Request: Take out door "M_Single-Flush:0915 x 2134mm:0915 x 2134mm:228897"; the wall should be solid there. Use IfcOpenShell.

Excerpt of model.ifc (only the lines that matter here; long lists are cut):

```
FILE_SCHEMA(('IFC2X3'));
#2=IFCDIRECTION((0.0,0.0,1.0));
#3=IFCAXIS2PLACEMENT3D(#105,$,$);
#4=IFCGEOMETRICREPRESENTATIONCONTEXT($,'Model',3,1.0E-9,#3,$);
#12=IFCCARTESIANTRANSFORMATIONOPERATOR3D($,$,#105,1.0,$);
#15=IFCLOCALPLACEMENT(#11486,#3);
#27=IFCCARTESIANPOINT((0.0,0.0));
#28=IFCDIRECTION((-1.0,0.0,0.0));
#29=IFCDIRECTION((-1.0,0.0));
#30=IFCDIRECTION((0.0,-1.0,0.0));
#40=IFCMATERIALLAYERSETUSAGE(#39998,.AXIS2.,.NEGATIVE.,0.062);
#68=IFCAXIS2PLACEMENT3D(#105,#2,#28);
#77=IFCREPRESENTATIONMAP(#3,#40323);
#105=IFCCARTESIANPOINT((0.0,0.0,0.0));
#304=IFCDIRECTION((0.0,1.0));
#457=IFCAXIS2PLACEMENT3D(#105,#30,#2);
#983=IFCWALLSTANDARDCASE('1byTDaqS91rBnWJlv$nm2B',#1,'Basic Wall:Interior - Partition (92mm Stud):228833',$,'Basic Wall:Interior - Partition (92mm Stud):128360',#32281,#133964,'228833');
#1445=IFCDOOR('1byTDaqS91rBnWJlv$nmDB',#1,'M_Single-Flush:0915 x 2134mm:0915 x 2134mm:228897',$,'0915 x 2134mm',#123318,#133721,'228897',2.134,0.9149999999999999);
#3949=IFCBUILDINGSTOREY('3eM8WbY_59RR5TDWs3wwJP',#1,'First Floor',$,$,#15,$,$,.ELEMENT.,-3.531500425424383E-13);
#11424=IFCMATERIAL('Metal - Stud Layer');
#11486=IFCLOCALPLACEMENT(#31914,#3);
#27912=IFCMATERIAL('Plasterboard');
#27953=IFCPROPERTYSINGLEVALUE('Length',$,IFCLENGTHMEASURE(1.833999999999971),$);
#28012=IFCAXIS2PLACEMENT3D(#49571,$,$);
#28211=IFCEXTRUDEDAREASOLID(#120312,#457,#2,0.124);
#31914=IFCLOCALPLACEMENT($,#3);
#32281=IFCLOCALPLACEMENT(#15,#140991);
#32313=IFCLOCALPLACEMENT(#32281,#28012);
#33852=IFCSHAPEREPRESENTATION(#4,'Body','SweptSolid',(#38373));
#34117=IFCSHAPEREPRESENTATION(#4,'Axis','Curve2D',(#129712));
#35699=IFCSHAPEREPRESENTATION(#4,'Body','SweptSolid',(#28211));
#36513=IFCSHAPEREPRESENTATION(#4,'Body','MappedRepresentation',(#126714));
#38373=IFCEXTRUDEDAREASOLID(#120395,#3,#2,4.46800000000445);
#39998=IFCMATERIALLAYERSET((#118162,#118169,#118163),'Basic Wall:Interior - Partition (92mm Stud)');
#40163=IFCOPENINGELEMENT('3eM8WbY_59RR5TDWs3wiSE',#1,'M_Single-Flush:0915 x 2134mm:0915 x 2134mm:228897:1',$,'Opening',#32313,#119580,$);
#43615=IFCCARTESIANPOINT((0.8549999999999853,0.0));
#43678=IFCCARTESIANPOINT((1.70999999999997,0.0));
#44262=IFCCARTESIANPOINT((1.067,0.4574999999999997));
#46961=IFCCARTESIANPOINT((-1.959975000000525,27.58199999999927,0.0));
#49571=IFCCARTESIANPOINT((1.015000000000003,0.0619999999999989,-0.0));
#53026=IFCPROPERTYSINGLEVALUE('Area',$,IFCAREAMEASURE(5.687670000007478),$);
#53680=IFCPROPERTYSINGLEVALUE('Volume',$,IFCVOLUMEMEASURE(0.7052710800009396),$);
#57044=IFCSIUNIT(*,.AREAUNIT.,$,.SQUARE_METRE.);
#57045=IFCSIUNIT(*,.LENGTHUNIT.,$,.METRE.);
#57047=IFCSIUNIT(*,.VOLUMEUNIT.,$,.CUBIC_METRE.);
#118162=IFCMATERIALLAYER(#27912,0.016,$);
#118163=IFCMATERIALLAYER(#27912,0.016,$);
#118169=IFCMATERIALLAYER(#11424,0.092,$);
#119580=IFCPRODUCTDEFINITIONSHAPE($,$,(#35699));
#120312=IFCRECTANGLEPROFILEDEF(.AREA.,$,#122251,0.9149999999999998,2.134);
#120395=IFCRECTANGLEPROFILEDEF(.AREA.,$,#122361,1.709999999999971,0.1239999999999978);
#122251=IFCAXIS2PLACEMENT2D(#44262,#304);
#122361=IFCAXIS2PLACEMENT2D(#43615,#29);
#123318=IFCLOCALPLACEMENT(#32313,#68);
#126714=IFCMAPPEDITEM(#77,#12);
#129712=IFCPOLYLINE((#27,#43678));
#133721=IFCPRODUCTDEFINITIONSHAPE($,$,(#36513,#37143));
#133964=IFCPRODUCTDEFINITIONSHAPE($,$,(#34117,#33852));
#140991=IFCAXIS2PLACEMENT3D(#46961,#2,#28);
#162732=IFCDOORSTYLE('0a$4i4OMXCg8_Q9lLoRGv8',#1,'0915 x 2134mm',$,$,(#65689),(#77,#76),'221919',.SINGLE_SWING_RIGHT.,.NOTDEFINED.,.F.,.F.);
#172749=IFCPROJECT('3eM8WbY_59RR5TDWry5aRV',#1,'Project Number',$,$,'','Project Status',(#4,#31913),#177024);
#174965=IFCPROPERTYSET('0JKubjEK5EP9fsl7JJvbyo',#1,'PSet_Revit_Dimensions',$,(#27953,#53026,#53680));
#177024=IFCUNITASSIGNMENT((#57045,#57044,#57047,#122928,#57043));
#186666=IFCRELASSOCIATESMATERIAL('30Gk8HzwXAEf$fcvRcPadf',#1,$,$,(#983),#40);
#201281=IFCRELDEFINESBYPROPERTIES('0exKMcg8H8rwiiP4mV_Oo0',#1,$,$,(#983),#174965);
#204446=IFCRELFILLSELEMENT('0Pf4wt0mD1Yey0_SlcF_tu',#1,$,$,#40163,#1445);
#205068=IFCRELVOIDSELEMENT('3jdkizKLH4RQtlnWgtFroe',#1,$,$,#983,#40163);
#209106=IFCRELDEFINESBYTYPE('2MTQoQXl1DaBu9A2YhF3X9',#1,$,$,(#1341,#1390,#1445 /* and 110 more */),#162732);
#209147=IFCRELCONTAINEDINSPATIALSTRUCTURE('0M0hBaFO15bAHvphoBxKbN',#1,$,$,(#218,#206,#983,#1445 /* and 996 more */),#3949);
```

```python
import ifcopenshell
import ifcopenshell.api.feature
import ifcopenshell.api.pset
import ifcopenshell.api.root
import ifcopenshell.geom
import ifcopenshell.util.element
import ifcopenshell.util.shape
import ifcopenshell.util.unit

model = ifcopenshell.open("model.ifc")
area_scale = ifcopenshell.util.unit.calculate_unit_scale(model, "AREAUNIT")
volume_scale = ifcopenshell.util.unit.calculate_unit_scale(model, "VOLUMEUNIT")
settings = ifcopenshell.geom.settings()


def volume(element):
    """Net volume in cubic metres, openings subtracted."""
    shape = ifcopenshell.geom.create_shape(settings, element)
    return ifcopenshell.util.shape.get_volume(shape.geometry)


door = model.by_id(1445)
opening = door.FillsVoids[0].RelatingOpeningElement
wall = opening.VoidsElements[0].RelatingBuildingElement
before = volume(wall)

ifcopenshell.api.root.remove_product(model, product=door)
ifcopenshell.api.feature.remove_feature(model, feature=opening)

after = volume(wall)
thickness = 0.124  # wall thickness in metres

# Update the wall's stored quantities.
pset = model.by_id(ifcopenshell.util.element.get_pset(wall, "PSet_Revit_Dimensions", should_inherit=False)["id"])
ifcopenshell.api.pset.edit_pset(model, pset=pset, properties={
    "Area": model.create_entity("IfcAreaMeasure", after / thickness / area_scale),
    "Volume": model.create_entity("IfcVolumeMeasure", after / volume_scale),
})

print(f"wall volume {before:.3f} -> {after:.3f} m3")

model.write("model_updated.ifc")
```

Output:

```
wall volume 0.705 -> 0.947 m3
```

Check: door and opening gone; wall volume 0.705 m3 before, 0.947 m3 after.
